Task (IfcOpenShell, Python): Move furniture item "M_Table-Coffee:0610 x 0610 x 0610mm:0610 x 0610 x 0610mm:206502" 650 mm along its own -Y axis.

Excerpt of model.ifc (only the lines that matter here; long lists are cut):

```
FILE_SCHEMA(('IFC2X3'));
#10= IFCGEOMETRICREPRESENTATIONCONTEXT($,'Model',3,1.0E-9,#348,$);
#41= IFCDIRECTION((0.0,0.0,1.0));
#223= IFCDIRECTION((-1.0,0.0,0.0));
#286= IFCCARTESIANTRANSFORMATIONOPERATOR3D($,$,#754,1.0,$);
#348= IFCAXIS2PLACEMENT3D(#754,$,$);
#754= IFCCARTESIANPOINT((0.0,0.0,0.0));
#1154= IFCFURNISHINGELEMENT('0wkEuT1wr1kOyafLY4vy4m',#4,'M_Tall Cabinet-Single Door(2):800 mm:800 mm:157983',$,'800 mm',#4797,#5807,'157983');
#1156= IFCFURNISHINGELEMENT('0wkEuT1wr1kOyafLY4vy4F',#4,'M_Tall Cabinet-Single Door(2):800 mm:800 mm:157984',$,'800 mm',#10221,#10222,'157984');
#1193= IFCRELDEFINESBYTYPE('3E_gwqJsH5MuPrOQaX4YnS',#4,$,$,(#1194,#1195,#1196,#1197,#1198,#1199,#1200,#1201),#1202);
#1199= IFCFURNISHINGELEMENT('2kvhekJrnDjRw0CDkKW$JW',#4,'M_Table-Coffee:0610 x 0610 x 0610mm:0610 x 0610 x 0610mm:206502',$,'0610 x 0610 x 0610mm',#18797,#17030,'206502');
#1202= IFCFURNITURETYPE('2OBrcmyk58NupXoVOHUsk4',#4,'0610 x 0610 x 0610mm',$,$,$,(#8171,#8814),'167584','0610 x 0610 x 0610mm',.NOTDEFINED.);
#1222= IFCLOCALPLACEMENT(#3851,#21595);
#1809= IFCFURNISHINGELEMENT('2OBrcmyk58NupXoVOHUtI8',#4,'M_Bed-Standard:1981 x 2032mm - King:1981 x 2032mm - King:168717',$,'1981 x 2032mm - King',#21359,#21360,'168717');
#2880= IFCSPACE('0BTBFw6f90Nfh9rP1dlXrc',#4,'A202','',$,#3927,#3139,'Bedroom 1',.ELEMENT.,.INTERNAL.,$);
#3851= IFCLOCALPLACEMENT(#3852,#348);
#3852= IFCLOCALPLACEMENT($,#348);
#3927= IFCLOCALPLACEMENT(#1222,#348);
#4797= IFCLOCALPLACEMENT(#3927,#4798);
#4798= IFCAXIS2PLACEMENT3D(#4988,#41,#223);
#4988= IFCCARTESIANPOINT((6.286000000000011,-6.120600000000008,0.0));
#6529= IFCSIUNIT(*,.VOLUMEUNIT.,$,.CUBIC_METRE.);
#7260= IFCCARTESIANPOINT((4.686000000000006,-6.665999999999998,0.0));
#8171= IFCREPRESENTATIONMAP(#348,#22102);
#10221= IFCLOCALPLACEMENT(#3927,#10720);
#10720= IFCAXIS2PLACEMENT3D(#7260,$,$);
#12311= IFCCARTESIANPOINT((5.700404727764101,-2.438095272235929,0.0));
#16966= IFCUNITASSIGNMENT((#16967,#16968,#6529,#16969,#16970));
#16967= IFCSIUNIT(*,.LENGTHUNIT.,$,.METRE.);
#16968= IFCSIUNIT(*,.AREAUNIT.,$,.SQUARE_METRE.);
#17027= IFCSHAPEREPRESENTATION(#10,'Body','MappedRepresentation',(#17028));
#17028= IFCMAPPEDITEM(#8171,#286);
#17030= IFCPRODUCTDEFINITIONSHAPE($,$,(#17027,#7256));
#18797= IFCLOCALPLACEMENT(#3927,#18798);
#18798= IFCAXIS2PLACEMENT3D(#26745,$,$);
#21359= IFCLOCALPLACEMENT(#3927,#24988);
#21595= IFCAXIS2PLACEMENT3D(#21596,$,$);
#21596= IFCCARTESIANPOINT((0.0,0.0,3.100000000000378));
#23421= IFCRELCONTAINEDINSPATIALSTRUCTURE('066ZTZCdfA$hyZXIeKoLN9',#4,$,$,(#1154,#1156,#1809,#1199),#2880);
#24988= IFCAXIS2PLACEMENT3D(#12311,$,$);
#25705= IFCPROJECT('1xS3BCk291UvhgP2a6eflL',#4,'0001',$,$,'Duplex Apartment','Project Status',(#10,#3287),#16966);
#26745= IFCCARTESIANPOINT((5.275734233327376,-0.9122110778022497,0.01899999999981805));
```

```python
import ifcopenshell
import ifcopenshell.api.geometry
import ifcopenshell.util.placement

model = ifcopenshell.open("model.ifc")

item = model.by_guid("2kvhekJrnDjRw0CDkKW$JW")
matrix = ifcopenshell.util.placement.get_local_placement(item.ObjectPlacement)
matrix[:3, 3] -= matrix[:3, 1] * 0.65
ifcopenshell.api.geometry.edit_object_placement(model, product=item, matrix=matrix, is_si=False)

print(ifcopenshell.util.placement.get_local_placement(item.ObjectPlacement).round(3) + 0.0)

model.write("model-out.ifc")
```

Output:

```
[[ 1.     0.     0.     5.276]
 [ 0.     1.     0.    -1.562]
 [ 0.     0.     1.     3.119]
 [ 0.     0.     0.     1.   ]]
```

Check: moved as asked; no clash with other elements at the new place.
